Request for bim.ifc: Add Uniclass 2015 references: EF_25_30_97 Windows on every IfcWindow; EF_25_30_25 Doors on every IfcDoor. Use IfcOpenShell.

First a look at what the model holds.

```python
import ifcopenshell

model = ifcopenshell.open("bim.ifc")
print(model.schema)
print("classifications:", [c.Name for c in model.by_type("IfcClassification")])
for ifc_class in ("IfcDoor", "IfcRoof", "IfcStair", "IfcWall", "IfcWindow"):
    print(ifc_class, len(model.by_type(ifc_class)))
```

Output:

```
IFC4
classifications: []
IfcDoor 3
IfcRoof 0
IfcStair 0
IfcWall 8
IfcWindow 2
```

```python
import ifcopenshell
import ifcopenshell.api.classification

model = ifcopenshell.open("bim.ifc")

system = ifcopenshell.api.classification.add_classification(model, classification="Uniclass 2015")

codes = {
    "IfcWindow": ("EF_25_30_97", "Windows"),
    "IfcDoor": ("EF_25_30_25", "Doors"),
}
for ifc_class, (code, name) in codes.items():
    products = model.by_type(ifc_class)
    ifcopenshell.api.classification.add_reference(
        model, products=products, classification=system, identification=code, name=name
    )
    print(code, len(products))

model.write("bim_updated.ifc")
```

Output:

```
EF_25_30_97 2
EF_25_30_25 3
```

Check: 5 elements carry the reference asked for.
